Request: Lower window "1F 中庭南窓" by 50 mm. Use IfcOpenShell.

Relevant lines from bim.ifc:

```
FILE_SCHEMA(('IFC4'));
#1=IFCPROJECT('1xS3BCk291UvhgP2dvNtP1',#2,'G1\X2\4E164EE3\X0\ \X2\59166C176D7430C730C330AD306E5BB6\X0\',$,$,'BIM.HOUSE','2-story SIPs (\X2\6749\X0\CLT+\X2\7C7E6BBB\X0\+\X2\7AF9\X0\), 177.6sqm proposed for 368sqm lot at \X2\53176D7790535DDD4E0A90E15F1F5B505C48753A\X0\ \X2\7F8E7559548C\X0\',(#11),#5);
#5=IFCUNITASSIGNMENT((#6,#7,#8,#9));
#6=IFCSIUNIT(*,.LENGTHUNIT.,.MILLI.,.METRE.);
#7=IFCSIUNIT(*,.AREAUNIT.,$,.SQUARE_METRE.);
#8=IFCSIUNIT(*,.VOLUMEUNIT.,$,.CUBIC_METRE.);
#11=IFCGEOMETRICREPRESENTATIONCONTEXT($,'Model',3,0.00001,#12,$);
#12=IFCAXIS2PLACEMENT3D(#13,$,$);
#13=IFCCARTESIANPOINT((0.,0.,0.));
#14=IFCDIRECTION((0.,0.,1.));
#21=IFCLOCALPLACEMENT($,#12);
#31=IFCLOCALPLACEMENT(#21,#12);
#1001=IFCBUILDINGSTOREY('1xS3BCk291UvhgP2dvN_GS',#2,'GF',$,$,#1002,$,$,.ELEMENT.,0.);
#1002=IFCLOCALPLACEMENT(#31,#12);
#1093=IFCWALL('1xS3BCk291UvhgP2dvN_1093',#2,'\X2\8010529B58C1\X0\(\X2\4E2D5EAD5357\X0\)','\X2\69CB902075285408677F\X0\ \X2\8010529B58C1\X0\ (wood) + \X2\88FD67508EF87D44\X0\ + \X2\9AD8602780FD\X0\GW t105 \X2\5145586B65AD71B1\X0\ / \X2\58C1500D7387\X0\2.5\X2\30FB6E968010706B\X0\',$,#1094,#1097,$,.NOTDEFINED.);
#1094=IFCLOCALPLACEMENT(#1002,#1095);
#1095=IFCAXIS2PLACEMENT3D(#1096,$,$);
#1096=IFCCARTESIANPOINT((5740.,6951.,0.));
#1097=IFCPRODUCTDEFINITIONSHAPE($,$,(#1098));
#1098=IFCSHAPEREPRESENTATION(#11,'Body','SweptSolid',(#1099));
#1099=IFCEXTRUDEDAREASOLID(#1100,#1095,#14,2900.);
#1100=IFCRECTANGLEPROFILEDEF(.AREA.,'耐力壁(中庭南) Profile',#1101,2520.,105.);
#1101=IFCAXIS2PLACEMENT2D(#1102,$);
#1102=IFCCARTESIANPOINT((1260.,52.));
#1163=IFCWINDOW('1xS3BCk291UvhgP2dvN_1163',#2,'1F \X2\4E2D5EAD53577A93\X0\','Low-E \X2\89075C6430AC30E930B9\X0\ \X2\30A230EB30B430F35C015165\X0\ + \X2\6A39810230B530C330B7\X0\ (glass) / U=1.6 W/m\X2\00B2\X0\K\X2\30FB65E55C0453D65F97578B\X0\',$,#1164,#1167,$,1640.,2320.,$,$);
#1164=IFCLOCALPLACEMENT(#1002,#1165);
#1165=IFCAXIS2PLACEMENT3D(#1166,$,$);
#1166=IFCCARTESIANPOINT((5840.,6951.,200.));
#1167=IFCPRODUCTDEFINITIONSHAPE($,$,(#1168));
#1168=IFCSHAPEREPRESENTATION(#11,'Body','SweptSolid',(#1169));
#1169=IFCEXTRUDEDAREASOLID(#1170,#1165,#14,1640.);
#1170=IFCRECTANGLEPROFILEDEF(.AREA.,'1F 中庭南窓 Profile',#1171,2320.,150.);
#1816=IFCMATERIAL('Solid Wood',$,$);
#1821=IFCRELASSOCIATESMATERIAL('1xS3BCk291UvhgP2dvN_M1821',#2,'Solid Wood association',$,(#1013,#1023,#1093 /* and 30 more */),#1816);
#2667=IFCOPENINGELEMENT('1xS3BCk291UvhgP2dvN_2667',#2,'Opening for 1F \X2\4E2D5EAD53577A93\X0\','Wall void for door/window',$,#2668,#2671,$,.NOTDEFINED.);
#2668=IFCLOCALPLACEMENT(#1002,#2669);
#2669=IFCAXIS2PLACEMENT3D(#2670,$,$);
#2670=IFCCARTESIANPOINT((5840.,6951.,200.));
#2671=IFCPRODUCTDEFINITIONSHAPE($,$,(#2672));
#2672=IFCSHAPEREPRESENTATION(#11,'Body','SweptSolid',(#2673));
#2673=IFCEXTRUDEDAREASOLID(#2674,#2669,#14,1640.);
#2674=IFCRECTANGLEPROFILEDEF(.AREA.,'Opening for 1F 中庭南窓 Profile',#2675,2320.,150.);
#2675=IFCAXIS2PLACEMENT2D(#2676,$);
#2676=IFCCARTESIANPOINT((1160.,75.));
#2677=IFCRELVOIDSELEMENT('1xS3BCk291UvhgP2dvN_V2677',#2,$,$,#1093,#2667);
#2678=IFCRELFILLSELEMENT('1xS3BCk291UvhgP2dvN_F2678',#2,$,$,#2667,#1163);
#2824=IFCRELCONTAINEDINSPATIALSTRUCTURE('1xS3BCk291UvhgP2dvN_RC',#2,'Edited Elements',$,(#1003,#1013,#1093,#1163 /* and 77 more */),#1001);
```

```python
import numpy as np
import ifcopenshell
import ifcopenshell.api.geometry
import ifcopenshell.util.placement
import ifcopenshell.util.unit

model = ifcopenshell.open("bim.ifc")
unit_scale = ifcopenshell.util.unit.calculate_unit_scale(model)

window = model.by_guid("1xS3BCk291UvhgP2dvN_1163")
opening = window.FillsVoids[0].RelatingOpeningElement
dz = -0.05 / unit_scale

shift = np.array([0.0, 0.0, dz])
# The window is not placed relative to its opening, so move both.
for product in (opening, window):
    matrix = ifcopenshell.util.placement.get_local_placement(product.ObjectPlacement)
    matrix[:3, 3] += shift
    ifcopenshell.api.geometry.edit_object_placement(model, product=product, matrix=matrix, is_si=False)

print(f"moved by {dz * unit_scale:+.3f} m")

model.write("bim_v2.ifc")
```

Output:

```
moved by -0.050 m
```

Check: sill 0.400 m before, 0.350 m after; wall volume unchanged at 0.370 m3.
